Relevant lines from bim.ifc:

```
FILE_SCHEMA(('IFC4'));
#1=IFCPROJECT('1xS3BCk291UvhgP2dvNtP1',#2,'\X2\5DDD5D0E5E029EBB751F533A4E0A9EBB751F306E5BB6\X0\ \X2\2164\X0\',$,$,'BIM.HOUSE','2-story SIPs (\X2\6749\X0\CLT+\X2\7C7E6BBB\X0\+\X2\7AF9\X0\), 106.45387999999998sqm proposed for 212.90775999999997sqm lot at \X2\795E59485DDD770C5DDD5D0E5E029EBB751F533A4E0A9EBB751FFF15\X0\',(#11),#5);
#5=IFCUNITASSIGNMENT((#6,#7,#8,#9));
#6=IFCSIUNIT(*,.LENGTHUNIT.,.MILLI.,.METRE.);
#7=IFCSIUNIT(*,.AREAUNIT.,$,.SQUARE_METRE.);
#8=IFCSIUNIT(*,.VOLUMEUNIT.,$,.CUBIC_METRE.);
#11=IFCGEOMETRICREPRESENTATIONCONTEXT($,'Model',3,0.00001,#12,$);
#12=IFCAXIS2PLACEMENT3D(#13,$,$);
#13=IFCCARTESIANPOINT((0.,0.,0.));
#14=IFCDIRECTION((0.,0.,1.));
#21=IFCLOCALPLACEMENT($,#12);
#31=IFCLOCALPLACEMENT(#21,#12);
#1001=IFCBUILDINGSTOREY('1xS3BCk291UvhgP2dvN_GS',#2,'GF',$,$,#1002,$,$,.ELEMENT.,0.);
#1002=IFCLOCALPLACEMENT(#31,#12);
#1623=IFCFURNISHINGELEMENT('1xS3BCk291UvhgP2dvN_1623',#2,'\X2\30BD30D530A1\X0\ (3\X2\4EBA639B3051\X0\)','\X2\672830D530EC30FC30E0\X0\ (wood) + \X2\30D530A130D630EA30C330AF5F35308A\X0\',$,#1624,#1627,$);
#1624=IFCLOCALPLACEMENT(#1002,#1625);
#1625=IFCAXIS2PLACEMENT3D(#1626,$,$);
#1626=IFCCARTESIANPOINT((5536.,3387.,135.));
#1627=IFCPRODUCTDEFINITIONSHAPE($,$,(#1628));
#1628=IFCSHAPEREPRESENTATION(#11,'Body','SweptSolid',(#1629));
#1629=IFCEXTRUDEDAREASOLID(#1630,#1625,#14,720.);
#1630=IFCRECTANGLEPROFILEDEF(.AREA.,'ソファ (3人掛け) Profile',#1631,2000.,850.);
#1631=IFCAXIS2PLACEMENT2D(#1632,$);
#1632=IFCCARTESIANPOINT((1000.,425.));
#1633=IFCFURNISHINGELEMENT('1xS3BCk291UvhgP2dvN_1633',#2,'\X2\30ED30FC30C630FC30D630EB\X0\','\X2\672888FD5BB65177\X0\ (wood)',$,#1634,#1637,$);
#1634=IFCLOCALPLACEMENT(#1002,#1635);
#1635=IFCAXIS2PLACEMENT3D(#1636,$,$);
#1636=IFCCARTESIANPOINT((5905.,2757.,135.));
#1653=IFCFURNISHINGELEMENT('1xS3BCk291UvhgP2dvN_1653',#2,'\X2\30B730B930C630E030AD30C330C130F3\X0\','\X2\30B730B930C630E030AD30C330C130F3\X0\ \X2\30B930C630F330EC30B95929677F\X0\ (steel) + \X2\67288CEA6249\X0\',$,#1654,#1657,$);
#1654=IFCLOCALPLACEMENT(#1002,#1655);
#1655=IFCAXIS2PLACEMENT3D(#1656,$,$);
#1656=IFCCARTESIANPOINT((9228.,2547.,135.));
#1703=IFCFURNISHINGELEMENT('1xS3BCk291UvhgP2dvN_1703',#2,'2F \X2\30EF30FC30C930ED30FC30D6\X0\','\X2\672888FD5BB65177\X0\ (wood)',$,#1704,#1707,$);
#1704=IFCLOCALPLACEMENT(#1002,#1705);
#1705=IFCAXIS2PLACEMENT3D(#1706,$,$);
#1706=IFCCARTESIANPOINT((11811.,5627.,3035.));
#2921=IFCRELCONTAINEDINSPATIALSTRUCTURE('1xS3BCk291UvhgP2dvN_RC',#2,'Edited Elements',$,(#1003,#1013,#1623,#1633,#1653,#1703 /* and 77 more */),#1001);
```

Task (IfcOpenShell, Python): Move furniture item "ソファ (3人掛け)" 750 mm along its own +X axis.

```python
import ifcopenshell
import ifcopenshell.api.geometry
import ifcopenshell.util.placement
import ifcopenshell.util.unit

model = ifcopenshell.open("bim.ifc")
unit_scale = ifcopenshell.util.unit.calculate_unit_scale(model)

item = model.by_guid("1xS3BCk291UvhgP2dvN_1623")
matrix = ifcopenshell.util.placement.get_local_placement(item.ObjectPlacement)
matrix[:3, 3] += matrix[:3, 0] * 0.75 / unit_scale
ifcopenshell.api.geometry.edit_object_placement(model, product=item, matrix=matrix, is_si=False)

print(ifcopenshell.util.placement.get_local_placement(item.ObjectPlacement).round(3) + 0.0)

model.write("bim_edited.ifc")
```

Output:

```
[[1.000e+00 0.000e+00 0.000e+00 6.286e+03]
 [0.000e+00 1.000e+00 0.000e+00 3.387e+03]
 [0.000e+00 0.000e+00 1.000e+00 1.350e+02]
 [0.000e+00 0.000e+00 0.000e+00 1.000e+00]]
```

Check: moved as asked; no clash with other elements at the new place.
